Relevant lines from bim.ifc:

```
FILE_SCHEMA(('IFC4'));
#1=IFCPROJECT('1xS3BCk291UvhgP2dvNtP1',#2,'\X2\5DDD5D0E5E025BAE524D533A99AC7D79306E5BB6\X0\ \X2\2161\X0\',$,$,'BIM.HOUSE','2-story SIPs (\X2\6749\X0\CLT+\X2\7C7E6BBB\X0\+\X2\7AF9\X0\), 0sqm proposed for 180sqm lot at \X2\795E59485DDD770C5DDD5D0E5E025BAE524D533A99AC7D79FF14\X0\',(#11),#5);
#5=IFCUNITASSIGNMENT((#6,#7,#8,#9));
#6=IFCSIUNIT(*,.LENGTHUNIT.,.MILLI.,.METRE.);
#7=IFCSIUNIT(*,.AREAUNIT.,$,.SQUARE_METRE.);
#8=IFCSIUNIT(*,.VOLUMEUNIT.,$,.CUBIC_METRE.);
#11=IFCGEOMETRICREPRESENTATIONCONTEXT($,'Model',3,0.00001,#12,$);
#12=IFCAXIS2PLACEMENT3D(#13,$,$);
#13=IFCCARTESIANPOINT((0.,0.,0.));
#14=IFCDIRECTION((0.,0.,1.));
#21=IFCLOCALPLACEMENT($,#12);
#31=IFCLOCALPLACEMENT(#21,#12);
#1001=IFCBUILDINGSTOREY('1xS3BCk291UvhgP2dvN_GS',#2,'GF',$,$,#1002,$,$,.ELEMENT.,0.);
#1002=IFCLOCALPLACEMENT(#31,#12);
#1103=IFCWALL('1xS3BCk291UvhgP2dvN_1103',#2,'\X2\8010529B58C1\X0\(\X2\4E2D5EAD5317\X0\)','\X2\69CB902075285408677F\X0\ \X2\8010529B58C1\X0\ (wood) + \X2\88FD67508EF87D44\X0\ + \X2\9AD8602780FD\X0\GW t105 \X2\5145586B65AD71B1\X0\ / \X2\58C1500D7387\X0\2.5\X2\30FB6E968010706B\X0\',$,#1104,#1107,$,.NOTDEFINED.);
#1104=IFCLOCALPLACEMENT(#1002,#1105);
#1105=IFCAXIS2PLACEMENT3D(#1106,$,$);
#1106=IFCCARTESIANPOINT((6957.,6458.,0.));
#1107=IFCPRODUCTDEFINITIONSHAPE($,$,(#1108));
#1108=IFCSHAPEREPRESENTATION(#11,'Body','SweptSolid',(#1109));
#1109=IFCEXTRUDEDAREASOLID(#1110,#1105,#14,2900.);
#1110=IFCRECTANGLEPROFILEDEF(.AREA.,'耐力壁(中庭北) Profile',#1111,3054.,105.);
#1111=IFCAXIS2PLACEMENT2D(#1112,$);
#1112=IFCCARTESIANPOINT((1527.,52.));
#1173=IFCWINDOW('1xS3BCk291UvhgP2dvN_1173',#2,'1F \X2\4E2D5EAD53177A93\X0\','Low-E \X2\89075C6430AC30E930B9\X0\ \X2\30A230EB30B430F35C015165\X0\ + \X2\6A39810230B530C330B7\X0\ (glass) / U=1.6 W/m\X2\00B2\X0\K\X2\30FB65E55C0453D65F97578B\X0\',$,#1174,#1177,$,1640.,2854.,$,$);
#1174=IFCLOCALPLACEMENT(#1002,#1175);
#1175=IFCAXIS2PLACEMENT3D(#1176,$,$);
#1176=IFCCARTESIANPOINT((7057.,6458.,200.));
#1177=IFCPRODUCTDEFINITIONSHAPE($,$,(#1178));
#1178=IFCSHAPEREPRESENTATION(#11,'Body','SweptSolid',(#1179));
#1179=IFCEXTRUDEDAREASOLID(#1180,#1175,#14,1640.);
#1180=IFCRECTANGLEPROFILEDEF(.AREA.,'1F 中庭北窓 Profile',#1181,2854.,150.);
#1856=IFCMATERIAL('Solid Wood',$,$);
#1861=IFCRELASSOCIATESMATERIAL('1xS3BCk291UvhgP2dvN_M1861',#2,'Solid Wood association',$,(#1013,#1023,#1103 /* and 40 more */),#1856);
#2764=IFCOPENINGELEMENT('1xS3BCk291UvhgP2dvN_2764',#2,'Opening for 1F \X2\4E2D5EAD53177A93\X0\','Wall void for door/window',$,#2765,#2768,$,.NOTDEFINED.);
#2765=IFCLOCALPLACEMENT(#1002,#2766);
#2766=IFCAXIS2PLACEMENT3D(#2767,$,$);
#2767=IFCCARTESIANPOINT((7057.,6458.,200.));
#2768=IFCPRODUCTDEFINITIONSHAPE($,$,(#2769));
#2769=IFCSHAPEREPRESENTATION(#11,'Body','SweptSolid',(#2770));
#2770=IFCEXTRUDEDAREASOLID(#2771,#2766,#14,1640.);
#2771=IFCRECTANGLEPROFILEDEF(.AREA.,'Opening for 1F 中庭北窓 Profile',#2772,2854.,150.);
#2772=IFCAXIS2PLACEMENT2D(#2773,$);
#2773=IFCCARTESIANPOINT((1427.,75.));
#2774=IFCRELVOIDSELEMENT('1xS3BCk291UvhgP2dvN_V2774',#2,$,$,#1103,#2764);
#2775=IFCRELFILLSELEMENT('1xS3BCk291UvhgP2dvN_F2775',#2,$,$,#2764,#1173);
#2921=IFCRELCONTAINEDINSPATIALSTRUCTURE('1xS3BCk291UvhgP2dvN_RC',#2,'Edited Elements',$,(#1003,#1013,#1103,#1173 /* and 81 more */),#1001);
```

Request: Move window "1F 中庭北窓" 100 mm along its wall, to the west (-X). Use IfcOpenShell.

```python
import ifcopenshell
import ifcopenshell.api.geometry
import ifcopenshell.util.placement
import ifcopenshell.util.unit

model = ifcopenshell.open("bim.ifc")
unit_scale = ifcopenshell.util.unit.calculate_unit_scale(model)

window = model.by_id(1173)
opening = window.FillsVoids[0].RelatingOpeningElement
wall = opening.VoidsElements[0].RelatingBuildingElement

wall_matrix = ifcopenshell.util.placement.get_local_placement(wall.ObjectPlacement)
shift = wall_matrix[:3, 0] * -0.1 / unit_scale
before = ifcopenshell.util.placement.get_local_placement(window.ObjectPlacement)[:3, 3].copy()

# The window is not placed relative to its opening, so move both.
for product in (opening, window):
    matrix = ifcopenshell.util.placement.get_local_placement(product.ObjectPlacement)
    matrix[:3, 3] += shift
    ifcopenshell.api.geometry.edit_object_placement(model, product=product, matrix=matrix, is_si=False)

after = ifcopenshell.util.placement.get_local_placement(window.ObjectPlacement)[:3, 3]
print("window moved by", (after - before).round(3) + 0.0)

model.write("bim_updated.ifc")
```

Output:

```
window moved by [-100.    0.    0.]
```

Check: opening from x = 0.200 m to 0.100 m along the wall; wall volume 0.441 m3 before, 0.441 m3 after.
